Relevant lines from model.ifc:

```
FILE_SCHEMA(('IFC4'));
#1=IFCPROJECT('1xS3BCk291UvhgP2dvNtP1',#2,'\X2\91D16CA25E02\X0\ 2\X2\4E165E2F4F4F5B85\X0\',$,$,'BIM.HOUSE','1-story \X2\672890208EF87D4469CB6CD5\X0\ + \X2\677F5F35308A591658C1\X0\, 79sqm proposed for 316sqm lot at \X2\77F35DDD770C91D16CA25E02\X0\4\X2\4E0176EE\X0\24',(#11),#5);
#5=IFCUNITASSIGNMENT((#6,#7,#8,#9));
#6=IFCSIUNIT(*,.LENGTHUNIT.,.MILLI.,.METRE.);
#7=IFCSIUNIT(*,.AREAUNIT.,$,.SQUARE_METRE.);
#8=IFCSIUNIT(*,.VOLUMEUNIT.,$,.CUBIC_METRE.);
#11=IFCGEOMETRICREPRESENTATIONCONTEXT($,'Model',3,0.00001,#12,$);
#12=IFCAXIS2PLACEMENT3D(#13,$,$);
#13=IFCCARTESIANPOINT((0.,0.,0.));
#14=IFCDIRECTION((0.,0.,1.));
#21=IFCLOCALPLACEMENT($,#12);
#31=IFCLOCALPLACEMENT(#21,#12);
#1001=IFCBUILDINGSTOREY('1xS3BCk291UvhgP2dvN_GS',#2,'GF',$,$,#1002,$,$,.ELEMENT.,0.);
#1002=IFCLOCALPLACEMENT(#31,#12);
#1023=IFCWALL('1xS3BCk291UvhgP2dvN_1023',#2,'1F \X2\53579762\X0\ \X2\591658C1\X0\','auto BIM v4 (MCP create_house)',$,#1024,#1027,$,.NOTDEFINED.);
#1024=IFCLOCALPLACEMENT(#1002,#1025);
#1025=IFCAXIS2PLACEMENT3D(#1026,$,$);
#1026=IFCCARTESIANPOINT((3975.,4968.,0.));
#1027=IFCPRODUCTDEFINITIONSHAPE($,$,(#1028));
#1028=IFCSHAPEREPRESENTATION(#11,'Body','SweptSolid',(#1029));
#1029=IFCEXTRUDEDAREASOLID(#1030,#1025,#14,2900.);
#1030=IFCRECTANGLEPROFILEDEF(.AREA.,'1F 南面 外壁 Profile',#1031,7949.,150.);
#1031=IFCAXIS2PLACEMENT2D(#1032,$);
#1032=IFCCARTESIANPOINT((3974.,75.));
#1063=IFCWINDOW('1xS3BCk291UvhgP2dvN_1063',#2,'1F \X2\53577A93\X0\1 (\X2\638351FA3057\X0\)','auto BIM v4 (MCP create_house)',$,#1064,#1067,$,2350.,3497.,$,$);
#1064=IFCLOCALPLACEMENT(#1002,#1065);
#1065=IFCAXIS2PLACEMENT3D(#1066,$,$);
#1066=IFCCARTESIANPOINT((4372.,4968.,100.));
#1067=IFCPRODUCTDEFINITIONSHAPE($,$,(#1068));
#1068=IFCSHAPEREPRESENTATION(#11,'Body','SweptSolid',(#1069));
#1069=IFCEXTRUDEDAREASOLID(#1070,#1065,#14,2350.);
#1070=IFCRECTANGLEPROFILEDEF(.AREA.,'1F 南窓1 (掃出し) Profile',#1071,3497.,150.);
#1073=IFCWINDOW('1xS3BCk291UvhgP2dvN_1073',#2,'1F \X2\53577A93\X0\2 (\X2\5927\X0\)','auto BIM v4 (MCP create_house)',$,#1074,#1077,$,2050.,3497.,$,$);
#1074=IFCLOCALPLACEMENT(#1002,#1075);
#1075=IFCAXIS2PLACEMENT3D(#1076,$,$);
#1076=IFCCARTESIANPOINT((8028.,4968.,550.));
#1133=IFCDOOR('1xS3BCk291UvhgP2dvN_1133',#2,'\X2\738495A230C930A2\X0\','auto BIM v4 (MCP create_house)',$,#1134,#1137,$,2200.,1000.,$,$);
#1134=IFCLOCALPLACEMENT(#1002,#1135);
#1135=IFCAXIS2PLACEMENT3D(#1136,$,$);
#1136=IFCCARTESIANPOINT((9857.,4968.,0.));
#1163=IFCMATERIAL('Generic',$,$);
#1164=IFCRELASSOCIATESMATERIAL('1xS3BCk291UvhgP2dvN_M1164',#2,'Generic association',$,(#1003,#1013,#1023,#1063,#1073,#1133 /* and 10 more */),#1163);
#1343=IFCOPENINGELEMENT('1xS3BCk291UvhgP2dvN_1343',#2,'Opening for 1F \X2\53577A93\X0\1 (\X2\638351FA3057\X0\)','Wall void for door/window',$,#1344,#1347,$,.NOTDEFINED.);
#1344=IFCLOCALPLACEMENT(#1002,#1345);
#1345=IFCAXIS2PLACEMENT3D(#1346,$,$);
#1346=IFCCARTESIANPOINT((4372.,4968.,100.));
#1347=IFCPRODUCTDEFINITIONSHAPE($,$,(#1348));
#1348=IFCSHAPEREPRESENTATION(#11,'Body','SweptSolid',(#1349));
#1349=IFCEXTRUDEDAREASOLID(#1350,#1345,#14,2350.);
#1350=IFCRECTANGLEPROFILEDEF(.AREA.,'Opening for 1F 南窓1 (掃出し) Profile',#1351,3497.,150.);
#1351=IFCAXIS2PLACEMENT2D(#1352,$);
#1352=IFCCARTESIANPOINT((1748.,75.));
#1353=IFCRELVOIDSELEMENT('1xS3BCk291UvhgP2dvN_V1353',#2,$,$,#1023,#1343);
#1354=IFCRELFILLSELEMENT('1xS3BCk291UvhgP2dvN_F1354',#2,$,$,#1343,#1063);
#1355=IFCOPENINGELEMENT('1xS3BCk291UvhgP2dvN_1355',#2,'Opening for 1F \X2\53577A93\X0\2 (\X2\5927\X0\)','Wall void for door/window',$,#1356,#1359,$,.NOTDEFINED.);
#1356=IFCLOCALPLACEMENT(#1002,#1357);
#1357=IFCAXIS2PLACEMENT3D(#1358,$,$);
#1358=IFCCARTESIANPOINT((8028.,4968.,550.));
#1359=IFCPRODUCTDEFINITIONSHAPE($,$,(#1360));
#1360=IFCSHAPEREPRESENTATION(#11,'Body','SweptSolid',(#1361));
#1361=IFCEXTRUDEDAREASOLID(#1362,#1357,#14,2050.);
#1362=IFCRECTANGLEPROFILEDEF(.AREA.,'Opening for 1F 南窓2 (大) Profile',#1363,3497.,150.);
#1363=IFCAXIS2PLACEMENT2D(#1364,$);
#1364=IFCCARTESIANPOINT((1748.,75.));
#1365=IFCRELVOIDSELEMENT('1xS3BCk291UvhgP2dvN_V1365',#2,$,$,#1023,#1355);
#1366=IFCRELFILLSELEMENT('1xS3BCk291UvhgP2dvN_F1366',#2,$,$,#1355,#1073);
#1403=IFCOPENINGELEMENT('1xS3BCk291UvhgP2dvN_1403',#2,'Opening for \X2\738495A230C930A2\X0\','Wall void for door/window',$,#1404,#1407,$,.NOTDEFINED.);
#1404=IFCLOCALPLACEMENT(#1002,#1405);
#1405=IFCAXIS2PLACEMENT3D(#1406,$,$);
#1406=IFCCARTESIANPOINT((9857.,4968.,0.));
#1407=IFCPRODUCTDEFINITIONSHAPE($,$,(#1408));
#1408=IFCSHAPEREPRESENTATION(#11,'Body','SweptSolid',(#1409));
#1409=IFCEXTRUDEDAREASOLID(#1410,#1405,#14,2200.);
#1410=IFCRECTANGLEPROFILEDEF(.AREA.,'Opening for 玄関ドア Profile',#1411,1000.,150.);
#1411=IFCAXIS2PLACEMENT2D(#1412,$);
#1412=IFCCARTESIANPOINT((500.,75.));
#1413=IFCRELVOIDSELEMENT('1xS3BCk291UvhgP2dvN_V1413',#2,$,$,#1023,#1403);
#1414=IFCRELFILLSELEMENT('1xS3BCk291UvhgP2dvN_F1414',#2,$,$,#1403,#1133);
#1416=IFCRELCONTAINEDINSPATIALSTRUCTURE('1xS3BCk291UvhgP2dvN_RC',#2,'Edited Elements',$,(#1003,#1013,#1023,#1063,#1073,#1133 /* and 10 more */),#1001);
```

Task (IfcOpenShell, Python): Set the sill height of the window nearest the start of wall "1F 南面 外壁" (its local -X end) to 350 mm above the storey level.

```python
import numpy as np
import ifcopenshell
import ifcopenshell.api.geometry
import ifcopenshell.geom
import ifcopenshell.util.element
import ifcopenshell.util.placement
import ifcopenshell.util.shape
import ifcopenshell.util.unit

model = ifcopenshell.open("model.ifc")
unit_scale = ifcopenshell.util.unit.calculate_unit_scale(model)

window = model.by_guid("1xS3BCk291UvhgP2dvN_1063")
opening = window.FillsVoids[0].RelatingOpeningElement
storey = ifcopenshell.util.element.get_container(window, ifc_class="IfcBuildingStorey")
level = ifcopenshell.util.placement.get_local_placement(storey.ObjectPlacement)[2, 3]

# The opening's origin need not be at the sill, so measure its lowest point.
shape = ifcopenshell.geom.create_shape(ifcopenshell.geom.settings(), opening)
bottom = ifcopenshell.util.shape.get_shape_bottom_elevation(shape, shape.geometry) / unit_scale
dz = level + 350.0 - bottom

shift = np.array([0.0, 0.0, dz])
# The window is not placed relative to its opening, so move both.
for product in (opening, window):
    matrix = ifcopenshell.util.placement.get_local_placement(product.ObjectPlacement)
    matrix[:3, 3] += shift
    ifcopenshell.api.geometry.edit_object_placement(model, product=product, matrix=matrix, is_si=False)

print(f"moved by {dz * unit_scale:+.3f} m")

model.write("model_rev.ifc")
```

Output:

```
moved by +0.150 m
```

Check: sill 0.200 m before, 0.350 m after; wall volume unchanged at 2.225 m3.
